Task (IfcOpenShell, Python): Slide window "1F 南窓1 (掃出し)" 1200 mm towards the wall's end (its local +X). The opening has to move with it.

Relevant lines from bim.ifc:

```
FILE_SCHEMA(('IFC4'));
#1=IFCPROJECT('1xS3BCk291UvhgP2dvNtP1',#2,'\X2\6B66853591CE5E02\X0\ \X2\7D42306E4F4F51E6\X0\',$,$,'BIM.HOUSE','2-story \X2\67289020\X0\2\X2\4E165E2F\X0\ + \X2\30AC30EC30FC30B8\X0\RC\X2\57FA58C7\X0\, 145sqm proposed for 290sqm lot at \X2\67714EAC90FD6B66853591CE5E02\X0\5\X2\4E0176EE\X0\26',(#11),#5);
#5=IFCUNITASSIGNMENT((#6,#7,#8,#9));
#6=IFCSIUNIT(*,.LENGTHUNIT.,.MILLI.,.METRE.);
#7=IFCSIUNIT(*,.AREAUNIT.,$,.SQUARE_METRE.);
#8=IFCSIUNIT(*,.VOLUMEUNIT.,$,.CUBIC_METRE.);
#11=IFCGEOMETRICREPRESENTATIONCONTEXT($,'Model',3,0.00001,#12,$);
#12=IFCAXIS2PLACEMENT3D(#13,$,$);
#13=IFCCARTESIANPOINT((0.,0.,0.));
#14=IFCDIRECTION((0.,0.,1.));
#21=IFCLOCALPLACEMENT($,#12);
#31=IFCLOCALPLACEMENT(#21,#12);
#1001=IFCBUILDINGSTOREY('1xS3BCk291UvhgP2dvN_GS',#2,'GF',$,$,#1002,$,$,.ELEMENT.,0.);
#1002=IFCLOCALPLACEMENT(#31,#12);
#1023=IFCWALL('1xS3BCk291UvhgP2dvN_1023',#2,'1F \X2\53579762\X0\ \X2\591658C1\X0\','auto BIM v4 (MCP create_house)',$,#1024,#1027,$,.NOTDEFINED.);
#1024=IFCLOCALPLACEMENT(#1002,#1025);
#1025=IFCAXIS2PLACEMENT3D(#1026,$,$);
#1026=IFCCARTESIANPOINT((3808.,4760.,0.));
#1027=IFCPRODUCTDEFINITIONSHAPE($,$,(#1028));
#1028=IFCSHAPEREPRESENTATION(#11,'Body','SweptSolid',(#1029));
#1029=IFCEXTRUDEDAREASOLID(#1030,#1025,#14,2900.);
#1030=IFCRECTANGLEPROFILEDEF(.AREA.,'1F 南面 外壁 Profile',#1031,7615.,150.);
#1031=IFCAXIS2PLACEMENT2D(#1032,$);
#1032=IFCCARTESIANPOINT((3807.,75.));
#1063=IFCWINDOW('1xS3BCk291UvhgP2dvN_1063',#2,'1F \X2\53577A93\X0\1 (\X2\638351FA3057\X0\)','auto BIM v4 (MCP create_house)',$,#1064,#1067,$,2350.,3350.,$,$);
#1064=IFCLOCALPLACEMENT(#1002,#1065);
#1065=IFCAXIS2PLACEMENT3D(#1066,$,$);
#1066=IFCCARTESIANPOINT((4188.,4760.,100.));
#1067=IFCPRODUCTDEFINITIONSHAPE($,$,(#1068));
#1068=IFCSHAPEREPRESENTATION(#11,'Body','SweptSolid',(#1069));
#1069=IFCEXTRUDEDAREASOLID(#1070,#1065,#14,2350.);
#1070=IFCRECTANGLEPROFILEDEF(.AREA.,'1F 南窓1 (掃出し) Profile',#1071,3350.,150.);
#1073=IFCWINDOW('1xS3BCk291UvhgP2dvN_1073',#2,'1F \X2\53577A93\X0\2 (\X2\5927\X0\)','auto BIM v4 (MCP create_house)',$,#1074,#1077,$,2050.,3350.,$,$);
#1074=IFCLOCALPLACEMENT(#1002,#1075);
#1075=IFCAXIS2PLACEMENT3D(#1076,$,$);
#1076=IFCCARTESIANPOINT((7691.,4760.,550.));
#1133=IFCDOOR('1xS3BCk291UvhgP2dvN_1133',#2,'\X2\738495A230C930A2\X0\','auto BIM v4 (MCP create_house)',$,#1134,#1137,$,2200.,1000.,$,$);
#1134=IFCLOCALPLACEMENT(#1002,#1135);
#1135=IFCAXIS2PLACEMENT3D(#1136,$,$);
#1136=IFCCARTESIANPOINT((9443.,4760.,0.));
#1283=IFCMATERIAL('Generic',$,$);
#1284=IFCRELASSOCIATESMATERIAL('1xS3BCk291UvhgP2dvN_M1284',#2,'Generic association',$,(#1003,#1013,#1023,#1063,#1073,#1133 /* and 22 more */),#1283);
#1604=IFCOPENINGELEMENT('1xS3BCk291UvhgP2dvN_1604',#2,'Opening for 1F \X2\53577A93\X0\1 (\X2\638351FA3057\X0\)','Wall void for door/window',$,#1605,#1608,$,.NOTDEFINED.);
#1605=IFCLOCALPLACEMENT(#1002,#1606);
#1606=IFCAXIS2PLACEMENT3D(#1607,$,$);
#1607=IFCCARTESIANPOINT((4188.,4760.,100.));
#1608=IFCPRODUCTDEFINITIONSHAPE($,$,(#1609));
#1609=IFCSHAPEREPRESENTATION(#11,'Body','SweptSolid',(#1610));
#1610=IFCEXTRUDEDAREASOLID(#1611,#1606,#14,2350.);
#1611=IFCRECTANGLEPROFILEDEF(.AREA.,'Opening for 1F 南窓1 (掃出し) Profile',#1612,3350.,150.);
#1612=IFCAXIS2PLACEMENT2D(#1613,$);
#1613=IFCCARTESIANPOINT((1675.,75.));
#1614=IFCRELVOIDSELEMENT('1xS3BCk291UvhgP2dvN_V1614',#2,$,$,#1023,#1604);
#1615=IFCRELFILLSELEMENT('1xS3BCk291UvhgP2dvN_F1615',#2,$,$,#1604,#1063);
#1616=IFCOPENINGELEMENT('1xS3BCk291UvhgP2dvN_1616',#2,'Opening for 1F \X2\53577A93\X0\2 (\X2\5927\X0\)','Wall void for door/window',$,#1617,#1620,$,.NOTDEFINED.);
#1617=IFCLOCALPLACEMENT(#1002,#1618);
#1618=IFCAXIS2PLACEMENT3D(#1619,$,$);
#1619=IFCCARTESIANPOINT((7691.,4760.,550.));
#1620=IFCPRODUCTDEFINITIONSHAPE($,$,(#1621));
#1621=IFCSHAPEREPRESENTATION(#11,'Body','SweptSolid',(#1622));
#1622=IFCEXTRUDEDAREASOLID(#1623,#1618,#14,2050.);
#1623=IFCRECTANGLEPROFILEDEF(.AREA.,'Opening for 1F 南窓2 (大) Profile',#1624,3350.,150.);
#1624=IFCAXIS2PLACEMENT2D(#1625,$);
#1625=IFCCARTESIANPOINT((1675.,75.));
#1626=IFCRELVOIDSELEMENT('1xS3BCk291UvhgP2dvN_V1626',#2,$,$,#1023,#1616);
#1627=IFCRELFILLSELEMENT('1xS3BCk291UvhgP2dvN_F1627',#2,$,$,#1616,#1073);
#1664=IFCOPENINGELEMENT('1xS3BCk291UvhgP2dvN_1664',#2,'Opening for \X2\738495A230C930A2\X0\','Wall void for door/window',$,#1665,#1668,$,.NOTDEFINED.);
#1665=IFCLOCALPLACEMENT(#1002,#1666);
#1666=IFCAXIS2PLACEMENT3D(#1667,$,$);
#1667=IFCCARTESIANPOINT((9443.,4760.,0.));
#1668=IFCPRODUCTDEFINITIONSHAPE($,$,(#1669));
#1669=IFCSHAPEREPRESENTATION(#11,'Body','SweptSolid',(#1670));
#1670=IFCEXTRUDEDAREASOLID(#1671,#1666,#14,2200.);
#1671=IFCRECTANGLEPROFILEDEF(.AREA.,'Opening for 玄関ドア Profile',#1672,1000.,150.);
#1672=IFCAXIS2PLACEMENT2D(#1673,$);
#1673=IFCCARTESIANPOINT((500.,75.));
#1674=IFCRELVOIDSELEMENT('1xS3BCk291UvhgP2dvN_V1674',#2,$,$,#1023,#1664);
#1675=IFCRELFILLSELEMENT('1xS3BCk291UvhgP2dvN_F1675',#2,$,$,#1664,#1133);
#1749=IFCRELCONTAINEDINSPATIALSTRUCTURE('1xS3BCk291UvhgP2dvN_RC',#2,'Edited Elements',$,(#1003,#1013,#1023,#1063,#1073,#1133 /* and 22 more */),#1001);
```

```python
import ifcopenshell
import ifcopenshell.api.geometry
import ifcopenshell.util.placement

model = ifcopenshell.open("bim.ifc")

window = model.by_guid("1xS3BCk291UvhgP2dvN_1063")
opening = window.FillsVoids[0].RelatingOpeningElement
wall = opening.VoidsElements[0].RelatingBuildingElement

wall_matrix = ifcopenshell.util.placement.get_local_placement(wall.ObjectPlacement)
shift = wall_matrix[:3, 0] * 1200.0
before = ifcopenshell.util.placement.get_local_placement(window.ObjectPlacement)[:3, 3].copy()

# The window is not placed relative to its opening, so move both.
for product in (opening, window):
    matrix = ifcopenshell.util.placement.get_local_placement(product.ObjectPlacement)
    matrix[:3, 3] += shift
    ifcopenshell.api.geometry.edit_object_placement(model, product=product, matrix=matrix, is_si=False)

after = ifcopenshell.util.placement.get_local_placement(window.ObjectPlacement)[:3, 3]
print("window moved by", (after - before).round(3) + 0.0)

model.write("bim_updated.ifc")
```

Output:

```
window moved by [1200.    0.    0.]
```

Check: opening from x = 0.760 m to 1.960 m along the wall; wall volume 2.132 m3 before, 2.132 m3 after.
